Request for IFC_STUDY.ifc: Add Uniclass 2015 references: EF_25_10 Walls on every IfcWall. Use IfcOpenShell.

First a look at what the model holds.

```python
import ifcopenshell

model = ifcopenshell.open("IFC_STUDY.ifc")
print(model.schema)
print("classifications:", [c.Name for c in model.by_type("IfcClassification")])
for ifc_class in ("IfcDoor", "IfcRoof", "IfcStair", "IfcWall", "IfcWindow"):
    print(ifc_class, len(model.by_type(ifc_class)))
```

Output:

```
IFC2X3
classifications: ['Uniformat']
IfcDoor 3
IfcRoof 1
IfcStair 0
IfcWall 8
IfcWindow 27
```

```python
import ifcopenshell
import ifcopenshell.api.classification

model = ifcopenshell.open("IFC_STUDY.ifc")

# IFC2X3 requires Source and Edition and has no link from the project to the system.
system = model.create_entity("IfcClassification", Source="NBS", Edition="2015", Name="Uniclass 2015")

codes = {
    "IfcWall": ("EF_25_10", "Walls"),
}
for ifc_class, (code, name) in codes.items():
    products = model.by_type(ifc_class)
    ifcopenshell.api.classification.add_reference(
        model, products=products, classification=system, identification=code, name=name
    )
    print(code, len(products))

model.write("IFC_STUDY_updated.ifc")
```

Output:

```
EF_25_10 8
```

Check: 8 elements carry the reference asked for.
